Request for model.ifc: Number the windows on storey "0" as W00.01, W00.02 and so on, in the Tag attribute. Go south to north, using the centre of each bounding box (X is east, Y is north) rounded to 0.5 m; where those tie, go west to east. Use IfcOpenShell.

First a look at what the model holds.

```python
import ifcopenshell
import ifcopenshell.util.element
import ifcopenshell.util.placement

model = ifcopenshell.open("model.ifc")
print(model.schema)
storey = next(s for s in model.by_type("IfcBuildingStorey") if s.Name == "0")
windows = [e for e in ifcopenshell.util.element.get_decomposition(storey) if e.is_a("IfcWindow")]
for e in sorted(windows, key=lambda e: e.id()):
    origin = ifcopenshell.util.placement.get_local_placement(e.ObjectPlacement)[:3, 3]
    print(e.id(), e.Tag, e.Name, origin.round(2) + 0.0, sep=" | ")
```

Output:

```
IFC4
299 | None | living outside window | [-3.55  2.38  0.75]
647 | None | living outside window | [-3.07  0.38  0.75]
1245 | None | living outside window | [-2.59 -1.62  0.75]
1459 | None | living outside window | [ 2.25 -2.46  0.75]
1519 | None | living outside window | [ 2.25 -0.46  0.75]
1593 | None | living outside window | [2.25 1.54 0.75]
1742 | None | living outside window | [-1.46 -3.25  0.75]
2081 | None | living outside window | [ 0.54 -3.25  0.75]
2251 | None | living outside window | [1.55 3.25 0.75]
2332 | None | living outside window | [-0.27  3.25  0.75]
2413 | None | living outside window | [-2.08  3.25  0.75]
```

```python
import ifcopenshell
import ifcopenshell.geom
import ifcopenshell.util.element
import ifcopenshell.util.shape

model = ifcopenshell.open("model.ifc")
settings = ifcopenshell.geom.settings()
settings.set("use-world-coords", True)


def centre(element):
    shape = ifcopenshell.geom.create_shape(settings, element)
    return ifcopenshell.util.shape.get_bbox_centroid(shape.geometry)


storey = next(s for s in model.by_type("IfcBuildingStorey") if s.Name == "0")
windows = [e for e in ifcopenshell.util.element.get_decomposition(storey) if e.is_a("IfcWindow")]

# Insertion points can sit at a corner or the storey origin, so sort by the geometry (in metres).
centres = {e: centre(e) for e in windows}
windows.sort(key=lambda e: (round(centres[e][1] / 0.5), centres[e][0]))

for i, e in enumerate(windows, start=1):
    number = f"W00.{i:02d}"
    e.Tag = number
    print(e.id(), number)

model.write("model-out.ifc")
```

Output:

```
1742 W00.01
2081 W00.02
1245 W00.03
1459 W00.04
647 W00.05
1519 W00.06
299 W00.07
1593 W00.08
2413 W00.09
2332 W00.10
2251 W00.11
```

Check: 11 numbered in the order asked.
